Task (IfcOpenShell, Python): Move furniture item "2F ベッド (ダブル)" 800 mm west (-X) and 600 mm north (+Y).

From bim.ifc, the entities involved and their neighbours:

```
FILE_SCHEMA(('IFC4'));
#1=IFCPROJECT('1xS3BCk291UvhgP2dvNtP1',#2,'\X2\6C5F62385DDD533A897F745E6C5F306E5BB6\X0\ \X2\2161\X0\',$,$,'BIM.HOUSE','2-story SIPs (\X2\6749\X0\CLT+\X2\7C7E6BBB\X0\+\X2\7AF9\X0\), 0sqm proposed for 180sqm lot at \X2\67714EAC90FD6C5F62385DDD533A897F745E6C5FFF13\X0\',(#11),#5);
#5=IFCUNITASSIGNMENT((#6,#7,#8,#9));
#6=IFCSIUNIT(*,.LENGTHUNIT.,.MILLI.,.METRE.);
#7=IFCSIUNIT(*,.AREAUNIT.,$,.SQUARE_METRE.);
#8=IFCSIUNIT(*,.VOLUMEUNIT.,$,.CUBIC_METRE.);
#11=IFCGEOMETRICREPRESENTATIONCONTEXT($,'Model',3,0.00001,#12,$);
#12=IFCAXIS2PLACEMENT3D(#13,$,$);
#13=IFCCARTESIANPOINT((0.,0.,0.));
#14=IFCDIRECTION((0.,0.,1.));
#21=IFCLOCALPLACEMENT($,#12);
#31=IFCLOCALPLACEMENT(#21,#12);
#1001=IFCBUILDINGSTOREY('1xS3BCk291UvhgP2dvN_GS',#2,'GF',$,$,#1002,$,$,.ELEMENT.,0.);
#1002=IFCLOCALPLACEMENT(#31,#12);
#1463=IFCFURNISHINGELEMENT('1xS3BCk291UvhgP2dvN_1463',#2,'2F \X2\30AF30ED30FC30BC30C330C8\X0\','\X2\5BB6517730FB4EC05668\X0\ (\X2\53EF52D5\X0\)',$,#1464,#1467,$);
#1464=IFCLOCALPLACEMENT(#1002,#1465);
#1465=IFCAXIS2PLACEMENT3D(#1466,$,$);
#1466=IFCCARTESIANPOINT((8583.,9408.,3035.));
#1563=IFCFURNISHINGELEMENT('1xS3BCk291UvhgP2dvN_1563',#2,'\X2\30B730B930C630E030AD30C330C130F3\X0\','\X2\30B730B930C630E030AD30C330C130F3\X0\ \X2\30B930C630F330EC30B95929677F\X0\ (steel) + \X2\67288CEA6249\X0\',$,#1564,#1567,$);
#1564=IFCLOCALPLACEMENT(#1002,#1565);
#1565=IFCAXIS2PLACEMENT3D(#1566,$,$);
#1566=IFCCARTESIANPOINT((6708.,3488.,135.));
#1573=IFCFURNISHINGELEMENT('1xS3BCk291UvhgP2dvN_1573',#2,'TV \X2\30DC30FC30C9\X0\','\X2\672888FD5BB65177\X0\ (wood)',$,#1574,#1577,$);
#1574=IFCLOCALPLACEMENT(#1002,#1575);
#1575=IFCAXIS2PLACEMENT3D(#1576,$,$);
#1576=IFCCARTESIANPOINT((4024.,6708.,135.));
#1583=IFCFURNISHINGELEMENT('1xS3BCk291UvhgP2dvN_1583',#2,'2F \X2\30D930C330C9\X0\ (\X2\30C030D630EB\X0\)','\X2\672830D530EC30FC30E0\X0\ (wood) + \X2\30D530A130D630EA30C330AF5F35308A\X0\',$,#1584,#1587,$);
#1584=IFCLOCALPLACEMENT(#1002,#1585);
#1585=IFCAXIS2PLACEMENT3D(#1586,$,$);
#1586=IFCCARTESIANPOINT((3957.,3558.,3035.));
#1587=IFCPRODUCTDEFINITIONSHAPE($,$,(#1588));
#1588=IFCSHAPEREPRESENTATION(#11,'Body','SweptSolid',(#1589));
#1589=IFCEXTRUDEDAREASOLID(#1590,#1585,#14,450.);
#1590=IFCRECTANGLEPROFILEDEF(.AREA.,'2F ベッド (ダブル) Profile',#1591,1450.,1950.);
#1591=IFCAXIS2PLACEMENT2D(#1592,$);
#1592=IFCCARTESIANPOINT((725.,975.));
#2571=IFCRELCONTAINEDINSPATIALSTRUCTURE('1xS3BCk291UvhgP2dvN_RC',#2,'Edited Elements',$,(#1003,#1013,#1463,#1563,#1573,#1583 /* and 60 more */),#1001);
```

```python
import ifcopenshell
import ifcopenshell.api.geometry
import ifcopenshell.util.placement

model = ifcopenshell.open("bim.ifc")

item = model.by_guid("1xS3BCk291UvhgP2dvN_1583")
matrix = ifcopenshell.util.placement.get_local_placement(item.ObjectPlacement)
matrix[0, 3] -= 800.0
matrix[1, 3] += 600.0
ifcopenshell.api.geometry.edit_object_placement(model, product=item, matrix=matrix, is_si=False)

print(ifcopenshell.util.placement.get_local_placement(item.ObjectPlacement).round(3) + 0.0)

model.write("bim_edited.ifc")
```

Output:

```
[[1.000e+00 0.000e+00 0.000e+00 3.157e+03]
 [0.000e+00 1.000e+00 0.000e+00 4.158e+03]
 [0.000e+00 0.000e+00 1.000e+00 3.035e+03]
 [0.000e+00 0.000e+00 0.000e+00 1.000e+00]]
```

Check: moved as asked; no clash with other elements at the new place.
